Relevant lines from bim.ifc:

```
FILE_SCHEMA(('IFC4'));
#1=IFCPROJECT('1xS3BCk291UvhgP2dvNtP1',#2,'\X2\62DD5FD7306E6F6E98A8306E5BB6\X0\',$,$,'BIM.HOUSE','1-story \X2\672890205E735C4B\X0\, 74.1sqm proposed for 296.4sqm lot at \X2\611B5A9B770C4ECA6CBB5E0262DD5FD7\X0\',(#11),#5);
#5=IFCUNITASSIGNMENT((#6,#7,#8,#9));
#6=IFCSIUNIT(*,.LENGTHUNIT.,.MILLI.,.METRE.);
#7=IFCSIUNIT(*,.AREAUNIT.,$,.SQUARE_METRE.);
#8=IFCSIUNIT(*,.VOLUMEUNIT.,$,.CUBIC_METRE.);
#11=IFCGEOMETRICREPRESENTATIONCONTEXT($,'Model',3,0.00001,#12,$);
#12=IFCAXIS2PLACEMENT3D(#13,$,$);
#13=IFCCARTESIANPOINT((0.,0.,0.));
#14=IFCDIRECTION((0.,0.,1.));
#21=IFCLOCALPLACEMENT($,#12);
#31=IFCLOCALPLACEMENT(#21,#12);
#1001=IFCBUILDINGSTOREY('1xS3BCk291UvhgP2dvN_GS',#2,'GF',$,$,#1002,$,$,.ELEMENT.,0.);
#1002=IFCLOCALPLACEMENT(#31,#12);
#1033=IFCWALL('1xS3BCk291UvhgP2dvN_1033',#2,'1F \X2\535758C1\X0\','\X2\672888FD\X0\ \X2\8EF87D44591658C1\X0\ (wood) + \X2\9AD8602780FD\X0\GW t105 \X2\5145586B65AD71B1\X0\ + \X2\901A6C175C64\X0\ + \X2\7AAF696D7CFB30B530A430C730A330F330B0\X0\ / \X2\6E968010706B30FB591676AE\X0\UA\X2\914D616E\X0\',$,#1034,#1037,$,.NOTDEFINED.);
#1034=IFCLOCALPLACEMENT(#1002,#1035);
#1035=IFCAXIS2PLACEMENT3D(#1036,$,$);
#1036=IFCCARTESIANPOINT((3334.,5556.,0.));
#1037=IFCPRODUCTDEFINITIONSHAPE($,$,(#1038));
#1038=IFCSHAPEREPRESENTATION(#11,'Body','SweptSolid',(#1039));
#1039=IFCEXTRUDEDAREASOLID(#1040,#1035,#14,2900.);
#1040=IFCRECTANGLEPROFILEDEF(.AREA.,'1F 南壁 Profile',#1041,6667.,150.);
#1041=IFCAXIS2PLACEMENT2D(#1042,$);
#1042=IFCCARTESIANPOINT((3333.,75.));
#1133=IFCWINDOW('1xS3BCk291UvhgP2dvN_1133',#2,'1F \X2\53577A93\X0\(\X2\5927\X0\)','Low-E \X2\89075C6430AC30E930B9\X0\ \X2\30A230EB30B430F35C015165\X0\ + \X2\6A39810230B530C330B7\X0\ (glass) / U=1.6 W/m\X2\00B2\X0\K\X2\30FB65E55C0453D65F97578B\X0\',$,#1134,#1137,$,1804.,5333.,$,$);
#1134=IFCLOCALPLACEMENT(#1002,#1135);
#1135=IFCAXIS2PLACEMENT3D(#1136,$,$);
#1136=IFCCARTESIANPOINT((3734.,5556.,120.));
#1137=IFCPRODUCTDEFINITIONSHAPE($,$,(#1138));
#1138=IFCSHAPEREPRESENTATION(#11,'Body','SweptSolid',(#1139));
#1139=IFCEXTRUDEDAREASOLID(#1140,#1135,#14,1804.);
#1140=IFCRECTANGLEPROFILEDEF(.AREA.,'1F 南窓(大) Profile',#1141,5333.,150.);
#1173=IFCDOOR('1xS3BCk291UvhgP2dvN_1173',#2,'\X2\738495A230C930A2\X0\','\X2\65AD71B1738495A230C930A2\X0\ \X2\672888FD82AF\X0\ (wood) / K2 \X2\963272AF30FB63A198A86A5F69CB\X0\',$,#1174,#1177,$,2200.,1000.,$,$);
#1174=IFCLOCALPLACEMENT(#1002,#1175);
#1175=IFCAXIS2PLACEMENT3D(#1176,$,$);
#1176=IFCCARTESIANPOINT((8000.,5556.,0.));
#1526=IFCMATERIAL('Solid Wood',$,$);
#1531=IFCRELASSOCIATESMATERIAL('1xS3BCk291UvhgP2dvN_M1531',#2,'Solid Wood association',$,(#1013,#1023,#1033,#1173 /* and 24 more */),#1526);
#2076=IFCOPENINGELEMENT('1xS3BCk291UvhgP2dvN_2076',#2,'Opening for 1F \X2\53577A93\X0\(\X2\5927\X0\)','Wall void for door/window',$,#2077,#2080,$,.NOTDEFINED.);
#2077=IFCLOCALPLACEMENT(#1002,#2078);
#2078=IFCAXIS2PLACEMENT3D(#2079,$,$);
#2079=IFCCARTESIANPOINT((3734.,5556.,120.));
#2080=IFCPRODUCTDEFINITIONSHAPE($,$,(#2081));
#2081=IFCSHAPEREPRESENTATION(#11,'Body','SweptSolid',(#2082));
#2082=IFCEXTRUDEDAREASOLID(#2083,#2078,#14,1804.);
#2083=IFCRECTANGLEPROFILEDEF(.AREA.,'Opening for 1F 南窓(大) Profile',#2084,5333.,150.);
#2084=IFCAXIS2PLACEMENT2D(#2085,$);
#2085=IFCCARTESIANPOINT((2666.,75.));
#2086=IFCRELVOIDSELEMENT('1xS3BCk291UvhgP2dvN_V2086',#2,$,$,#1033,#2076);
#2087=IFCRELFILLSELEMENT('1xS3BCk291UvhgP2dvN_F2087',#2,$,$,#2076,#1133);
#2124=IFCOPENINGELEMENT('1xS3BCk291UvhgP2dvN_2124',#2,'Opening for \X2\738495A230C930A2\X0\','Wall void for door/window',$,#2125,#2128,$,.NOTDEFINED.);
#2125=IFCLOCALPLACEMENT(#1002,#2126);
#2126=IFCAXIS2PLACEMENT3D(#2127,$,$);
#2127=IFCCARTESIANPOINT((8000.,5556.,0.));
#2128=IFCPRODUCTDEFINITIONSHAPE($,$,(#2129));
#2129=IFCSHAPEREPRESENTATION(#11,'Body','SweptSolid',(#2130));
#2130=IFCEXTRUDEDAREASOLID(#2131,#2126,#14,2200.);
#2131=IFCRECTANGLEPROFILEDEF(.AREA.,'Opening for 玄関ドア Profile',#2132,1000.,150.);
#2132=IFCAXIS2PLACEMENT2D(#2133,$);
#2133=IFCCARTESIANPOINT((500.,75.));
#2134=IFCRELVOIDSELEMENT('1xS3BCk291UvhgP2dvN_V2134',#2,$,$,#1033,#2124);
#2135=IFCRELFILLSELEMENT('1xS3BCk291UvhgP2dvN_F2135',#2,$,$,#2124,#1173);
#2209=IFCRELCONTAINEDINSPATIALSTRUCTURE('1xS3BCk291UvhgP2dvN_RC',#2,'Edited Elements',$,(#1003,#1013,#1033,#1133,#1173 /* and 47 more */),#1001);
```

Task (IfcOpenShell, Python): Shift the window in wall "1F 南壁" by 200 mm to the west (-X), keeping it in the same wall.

```python
import ifcopenshell
import ifcopenshell.api.geometry
import ifcopenshell.util.placement
import ifcopenshell.util.unit

model = ifcopenshell.open("bim.ifc")
unit_scale = ifcopenshell.util.unit.calculate_unit_scale(model)

window = model.by_id(1133)
opening = window.FillsVoids[0].RelatingOpeningElement
wall = opening.VoidsElements[0].RelatingBuildingElement

wall_matrix = ifcopenshell.util.placement.get_local_placement(wall.ObjectPlacement)
shift = wall_matrix[:3, 0] * -0.2 / unit_scale
before = ifcopenshell.util.placement.get_local_placement(window.ObjectPlacement)[:3, 3].copy()

# The window is not placed relative to its opening, so move both.
for product in (opening, window):
    matrix = ifcopenshell.util.placement.get_local_placement(product.ObjectPlacement)
    matrix[:3, 3] += shift
    ifcopenshell.api.geometry.edit_object_placement(model, product=product, matrix=matrix, is_si=False)

after = ifcopenshell.util.placement.get_local_placement(window.ObjectPlacement)[:3, 3]
print("window moved by", (after - before).round(3) + 0.0)

model.write("bim-out.ifc")
```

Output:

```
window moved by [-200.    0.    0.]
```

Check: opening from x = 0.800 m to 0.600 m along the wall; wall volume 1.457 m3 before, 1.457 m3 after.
